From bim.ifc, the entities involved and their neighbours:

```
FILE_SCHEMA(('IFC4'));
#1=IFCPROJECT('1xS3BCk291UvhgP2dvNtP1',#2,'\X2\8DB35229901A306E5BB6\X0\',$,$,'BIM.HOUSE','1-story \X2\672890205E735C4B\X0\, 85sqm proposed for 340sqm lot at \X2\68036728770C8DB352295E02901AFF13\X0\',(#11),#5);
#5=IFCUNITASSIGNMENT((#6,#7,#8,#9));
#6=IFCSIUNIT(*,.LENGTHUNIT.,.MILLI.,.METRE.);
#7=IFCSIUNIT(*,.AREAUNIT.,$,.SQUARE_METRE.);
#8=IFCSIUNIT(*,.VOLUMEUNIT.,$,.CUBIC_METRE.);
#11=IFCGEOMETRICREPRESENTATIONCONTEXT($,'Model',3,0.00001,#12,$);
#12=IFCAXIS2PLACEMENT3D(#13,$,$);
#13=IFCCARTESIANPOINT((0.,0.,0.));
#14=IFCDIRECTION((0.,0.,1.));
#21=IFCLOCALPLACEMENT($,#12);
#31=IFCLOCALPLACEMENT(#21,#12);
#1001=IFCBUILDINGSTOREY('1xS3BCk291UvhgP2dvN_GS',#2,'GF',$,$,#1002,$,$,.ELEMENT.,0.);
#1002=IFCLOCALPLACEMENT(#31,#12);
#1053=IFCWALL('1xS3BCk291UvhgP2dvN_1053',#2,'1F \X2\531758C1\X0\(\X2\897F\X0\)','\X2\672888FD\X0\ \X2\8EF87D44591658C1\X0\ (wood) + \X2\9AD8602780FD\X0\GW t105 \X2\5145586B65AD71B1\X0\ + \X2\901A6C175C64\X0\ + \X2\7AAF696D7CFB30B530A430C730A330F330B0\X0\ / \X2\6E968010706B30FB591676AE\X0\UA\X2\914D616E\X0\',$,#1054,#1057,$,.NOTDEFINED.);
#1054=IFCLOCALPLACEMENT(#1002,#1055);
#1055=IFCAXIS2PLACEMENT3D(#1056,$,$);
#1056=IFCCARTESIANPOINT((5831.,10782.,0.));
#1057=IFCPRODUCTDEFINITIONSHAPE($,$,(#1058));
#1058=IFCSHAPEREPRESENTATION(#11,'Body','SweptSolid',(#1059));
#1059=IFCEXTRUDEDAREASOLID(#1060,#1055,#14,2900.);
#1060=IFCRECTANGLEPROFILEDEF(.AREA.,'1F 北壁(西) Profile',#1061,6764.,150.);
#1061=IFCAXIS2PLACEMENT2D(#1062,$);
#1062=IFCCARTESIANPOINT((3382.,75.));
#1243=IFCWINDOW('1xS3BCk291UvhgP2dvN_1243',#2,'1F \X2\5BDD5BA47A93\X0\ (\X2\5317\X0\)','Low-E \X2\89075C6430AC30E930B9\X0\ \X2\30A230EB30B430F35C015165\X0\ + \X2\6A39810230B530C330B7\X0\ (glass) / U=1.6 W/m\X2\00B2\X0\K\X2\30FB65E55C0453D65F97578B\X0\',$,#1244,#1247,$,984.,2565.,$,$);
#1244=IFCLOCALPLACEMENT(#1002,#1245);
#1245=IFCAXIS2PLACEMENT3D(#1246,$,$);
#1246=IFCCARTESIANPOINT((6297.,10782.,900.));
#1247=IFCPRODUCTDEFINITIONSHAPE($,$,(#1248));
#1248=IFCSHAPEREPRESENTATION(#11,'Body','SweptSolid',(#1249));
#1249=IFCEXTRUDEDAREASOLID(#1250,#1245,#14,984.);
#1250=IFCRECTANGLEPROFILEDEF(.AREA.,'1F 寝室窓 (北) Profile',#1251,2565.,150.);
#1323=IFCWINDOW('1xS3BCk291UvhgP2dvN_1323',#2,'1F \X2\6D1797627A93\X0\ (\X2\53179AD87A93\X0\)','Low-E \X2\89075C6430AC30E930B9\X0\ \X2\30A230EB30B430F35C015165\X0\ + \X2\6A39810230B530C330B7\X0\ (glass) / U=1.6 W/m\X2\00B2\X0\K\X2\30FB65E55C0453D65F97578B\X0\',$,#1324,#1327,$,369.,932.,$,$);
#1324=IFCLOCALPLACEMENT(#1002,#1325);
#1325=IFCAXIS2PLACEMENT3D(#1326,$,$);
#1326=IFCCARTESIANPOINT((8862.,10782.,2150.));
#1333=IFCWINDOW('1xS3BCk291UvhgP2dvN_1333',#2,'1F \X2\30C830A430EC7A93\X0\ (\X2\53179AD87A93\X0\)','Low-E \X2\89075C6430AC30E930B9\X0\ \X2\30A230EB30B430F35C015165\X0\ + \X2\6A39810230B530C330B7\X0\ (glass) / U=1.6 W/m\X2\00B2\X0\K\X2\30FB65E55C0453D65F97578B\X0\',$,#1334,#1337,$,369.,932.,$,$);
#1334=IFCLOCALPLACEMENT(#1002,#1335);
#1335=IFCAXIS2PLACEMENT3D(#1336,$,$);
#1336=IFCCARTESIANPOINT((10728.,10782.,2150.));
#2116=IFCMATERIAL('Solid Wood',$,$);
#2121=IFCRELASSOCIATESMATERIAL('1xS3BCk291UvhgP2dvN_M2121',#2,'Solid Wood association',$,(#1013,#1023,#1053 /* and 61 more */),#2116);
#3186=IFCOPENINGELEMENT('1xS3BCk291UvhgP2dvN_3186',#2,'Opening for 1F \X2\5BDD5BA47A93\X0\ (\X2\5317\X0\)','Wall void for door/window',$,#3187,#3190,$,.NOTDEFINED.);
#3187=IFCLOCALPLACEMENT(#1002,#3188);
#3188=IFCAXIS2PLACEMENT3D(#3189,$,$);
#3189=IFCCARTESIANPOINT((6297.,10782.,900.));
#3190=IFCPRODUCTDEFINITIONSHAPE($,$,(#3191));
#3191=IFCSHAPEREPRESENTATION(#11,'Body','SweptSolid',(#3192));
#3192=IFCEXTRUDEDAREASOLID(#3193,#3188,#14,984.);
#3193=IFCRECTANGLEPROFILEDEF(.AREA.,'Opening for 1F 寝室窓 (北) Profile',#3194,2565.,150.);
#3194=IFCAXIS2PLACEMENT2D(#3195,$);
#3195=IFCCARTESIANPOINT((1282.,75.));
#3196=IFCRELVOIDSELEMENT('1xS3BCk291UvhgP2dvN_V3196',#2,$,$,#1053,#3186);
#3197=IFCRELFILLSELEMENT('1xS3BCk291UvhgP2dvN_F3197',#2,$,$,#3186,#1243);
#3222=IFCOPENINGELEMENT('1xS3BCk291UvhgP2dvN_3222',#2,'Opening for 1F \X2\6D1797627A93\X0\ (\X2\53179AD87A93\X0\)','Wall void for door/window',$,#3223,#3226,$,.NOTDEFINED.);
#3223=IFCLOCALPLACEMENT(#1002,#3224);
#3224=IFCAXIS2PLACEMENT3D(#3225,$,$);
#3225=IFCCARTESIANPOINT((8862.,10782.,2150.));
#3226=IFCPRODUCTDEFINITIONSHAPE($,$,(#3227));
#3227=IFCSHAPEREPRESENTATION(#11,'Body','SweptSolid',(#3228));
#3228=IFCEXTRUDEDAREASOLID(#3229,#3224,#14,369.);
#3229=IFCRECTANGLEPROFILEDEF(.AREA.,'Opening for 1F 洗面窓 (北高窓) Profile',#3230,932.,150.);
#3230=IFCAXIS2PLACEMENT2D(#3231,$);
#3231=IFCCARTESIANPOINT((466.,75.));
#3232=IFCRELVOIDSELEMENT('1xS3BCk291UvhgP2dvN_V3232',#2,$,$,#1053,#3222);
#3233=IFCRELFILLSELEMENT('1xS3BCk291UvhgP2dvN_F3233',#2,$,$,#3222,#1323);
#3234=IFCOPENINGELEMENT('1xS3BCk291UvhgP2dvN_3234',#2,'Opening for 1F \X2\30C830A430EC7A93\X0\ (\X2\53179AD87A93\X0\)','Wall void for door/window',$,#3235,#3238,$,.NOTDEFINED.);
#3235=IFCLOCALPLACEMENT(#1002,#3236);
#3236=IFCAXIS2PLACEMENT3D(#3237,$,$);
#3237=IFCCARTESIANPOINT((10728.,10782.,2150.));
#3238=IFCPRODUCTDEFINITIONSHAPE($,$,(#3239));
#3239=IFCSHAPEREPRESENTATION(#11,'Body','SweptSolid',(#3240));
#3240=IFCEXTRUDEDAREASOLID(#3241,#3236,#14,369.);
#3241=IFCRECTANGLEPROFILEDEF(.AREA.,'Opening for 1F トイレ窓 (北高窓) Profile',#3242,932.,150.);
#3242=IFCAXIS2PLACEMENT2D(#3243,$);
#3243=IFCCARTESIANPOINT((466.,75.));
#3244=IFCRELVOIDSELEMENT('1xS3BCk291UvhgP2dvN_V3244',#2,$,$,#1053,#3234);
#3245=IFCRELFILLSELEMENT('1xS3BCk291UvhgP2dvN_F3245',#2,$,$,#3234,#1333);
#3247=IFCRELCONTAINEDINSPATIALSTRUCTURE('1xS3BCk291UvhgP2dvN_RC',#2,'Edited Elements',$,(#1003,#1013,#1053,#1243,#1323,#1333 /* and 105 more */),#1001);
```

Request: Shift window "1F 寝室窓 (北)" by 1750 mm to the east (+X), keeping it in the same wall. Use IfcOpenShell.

```python
import ifcopenshell
import ifcopenshell.api.geometry
import ifcopenshell.util.placement

model = ifcopenshell.open("bim.ifc")

window = model.by_id(1243)
opening = window.FillsVoids[0].RelatingOpeningElement
wall = opening.VoidsElements[0].RelatingBuildingElement

wall_matrix = ifcopenshell.util.placement.get_local_placement(wall.ObjectPlacement)
shift = wall_matrix[:3, 0] * 1750.0
before = ifcopenshell.util.placement.get_local_placement(window.ObjectPlacement)[:3, 3].copy()

# The window is not placed relative to its opening, so move both.
for product in (opening, window):
    matrix = ifcopenshell.util.placement.get_local_placement(product.ObjectPlacement)
    matrix[:3, 3] += shift
    ifcopenshell.api.geometry.edit_object_placement(model, product=product, matrix=matrix, is_si=False)

after = ifcopenshell.util.placement.get_local_placement(window.ObjectPlacement)[:3, 3]
print("window moved by", (after - before).round(3) + 0.0)

model.write("bim_edited.ifc")
```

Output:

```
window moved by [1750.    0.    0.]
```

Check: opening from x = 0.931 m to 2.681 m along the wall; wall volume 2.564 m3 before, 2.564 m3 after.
